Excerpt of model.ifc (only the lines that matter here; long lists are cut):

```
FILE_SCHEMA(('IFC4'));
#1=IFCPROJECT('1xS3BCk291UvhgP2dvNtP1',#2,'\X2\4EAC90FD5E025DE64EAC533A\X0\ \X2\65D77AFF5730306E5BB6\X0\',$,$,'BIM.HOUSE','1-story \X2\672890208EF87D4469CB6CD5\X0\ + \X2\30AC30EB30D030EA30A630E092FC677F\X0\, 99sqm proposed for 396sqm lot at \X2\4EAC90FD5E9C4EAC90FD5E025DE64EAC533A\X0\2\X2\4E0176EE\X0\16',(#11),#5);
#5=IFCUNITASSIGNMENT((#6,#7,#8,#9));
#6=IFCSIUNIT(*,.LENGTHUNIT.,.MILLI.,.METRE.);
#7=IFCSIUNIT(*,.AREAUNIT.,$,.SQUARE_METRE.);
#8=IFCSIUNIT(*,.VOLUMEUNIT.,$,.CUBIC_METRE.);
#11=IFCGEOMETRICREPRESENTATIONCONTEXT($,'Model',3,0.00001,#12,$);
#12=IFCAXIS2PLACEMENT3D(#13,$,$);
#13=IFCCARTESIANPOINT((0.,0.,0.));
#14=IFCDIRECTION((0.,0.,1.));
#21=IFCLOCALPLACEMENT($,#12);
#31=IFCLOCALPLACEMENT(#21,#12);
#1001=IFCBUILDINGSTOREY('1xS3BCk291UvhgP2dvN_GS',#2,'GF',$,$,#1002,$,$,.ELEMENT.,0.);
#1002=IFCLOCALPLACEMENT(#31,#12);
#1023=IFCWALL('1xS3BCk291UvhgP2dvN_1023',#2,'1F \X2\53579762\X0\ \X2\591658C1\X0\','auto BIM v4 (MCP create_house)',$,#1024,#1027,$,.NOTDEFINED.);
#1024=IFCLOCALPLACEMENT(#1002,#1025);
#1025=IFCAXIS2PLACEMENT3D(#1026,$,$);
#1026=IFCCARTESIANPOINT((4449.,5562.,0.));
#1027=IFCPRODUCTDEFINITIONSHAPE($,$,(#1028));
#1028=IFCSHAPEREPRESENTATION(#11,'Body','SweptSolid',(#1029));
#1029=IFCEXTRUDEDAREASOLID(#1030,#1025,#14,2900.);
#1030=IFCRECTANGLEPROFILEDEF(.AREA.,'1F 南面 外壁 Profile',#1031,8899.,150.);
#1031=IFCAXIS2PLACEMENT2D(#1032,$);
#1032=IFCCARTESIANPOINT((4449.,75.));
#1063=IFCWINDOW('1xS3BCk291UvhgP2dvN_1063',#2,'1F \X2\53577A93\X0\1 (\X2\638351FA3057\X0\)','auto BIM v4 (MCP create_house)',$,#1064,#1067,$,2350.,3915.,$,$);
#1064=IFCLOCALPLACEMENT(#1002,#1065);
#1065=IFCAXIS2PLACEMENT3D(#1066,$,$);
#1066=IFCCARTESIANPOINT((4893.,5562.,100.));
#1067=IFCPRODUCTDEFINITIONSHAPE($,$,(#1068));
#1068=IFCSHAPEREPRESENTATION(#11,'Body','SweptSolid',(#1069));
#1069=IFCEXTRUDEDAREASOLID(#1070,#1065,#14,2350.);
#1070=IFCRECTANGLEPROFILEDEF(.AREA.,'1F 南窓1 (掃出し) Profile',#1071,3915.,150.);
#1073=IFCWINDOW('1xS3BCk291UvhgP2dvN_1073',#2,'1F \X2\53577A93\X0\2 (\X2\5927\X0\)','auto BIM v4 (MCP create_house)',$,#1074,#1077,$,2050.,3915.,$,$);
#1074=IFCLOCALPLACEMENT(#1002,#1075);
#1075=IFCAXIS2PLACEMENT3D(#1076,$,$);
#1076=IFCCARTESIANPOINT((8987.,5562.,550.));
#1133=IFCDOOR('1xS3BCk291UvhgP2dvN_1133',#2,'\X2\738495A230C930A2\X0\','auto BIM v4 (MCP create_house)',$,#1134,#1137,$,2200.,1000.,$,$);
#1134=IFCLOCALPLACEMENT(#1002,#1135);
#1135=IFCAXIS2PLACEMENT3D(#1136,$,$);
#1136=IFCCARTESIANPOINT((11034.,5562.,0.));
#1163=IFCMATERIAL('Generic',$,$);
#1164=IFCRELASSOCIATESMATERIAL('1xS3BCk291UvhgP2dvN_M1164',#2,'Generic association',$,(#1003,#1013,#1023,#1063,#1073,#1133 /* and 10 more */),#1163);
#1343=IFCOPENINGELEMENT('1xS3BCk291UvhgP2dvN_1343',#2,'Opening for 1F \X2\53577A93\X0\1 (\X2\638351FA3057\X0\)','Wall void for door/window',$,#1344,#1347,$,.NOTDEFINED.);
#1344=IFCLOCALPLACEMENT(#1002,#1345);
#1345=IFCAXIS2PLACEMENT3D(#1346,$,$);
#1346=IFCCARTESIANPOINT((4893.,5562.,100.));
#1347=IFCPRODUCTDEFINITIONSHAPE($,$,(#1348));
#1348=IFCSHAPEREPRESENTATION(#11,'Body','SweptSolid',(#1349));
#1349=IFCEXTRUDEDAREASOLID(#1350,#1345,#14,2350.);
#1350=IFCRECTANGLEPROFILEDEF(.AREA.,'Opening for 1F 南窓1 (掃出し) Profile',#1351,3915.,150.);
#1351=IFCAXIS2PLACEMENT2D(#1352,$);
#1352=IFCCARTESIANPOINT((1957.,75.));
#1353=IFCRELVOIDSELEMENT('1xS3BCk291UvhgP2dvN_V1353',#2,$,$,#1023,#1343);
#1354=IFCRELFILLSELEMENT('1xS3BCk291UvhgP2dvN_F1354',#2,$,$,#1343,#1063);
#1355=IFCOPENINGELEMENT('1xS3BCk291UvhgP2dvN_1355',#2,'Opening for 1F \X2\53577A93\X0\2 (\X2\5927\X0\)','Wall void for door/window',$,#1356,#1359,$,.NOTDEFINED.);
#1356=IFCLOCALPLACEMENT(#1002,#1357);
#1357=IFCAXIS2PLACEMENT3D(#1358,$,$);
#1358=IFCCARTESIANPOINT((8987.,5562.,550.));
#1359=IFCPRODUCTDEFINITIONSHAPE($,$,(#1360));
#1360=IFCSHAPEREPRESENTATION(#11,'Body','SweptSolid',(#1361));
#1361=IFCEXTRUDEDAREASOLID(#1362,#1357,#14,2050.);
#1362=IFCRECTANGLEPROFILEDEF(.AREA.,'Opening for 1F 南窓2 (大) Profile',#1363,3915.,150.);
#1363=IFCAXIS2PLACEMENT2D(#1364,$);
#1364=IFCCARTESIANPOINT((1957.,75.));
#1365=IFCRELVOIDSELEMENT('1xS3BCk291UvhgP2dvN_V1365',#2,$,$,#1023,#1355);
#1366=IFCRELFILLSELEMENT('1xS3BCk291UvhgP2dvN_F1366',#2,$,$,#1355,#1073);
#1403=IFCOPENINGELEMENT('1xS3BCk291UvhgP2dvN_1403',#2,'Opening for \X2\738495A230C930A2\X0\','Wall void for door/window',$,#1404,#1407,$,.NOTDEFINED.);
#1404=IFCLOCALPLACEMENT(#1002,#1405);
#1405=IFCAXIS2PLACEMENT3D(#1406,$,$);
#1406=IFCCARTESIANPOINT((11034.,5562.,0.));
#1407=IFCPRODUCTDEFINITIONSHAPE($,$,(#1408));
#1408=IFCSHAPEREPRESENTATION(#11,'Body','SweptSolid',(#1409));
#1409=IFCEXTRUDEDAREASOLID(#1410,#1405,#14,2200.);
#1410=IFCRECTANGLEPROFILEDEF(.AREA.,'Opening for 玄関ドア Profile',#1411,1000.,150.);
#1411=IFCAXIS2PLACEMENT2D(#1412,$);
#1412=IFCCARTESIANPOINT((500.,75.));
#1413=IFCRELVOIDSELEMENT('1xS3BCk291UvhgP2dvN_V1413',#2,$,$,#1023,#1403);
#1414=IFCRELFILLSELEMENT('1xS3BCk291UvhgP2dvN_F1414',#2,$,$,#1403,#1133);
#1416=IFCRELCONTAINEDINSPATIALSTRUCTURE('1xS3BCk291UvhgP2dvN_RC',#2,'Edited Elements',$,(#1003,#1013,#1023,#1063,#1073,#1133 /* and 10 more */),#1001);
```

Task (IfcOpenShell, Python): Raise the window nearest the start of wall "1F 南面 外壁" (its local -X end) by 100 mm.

```python
import numpy as np
import ifcopenshell
import ifcopenshell.api.geometry
import ifcopenshell.util.placement
import ifcopenshell.util.unit

model = ifcopenshell.open("model.ifc")
unit_scale = ifcopenshell.util.unit.calculate_unit_scale(model)

window = model.by_guid("1xS3BCk291UvhgP2dvN_1063")
opening = window.FillsVoids[0].RelatingOpeningElement
dz = 100.0

shift = np.array([0.0, 0.0, dz])
# The window is not placed relative to its opening, so move both.
for product in (opening, window):
    matrix = ifcopenshell.util.placement.get_local_placement(product.ObjectPlacement)
    matrix[:3, 3] += shift
    ifcopenshell.api.geometry.edit_object_placement(model, product=product, matrix=matrix, is_si=False)

print(f"moved by {dz * unit_scale:+.3f} m")

model.write("model-out.ifc")
```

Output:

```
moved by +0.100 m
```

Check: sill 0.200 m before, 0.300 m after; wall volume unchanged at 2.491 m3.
